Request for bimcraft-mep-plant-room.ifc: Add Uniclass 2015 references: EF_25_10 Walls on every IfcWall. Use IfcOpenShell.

First a look at what the model holds.

```python
import ifcopenshell

model = ifcopenshell.open("bimcraft-mep-plant-room.ifc")
print(model.schema)
print("classifications:", [c.Name for c in model.by_type("IfcClassification")])
for ifc_class in ("IfcDoor", "IfcRoof", "IfcStair", "IfcWall", "IfcWindow"):
    print(ifc_class, len(model.by_type(ifc_class)))
```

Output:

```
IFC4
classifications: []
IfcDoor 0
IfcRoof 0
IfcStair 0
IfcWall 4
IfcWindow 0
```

```python
import ifcopenshell
import ifcopenshell.api.classification

model = ifcopenshell.open("bimcraft-mep-plant-room.ifc")

system = ifcopenshell.api.classification.add_classification(model, classification="Uniclass 2015")

codes = {
    "IfcWall": ("EF_25_10", "Walls"),
}
for ifc_class, (code, name) in codes.items():
    products = model.by_type(ifc_class)
    ifcopenshell.api.classification.add_reference(
        model, products=products, classification=system, identification=code, name=name
    )
    print(code, len(products))

model.write("bimcraft-mep-plant-room_updated.ifc")
```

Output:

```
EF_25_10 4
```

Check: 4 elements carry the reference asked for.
